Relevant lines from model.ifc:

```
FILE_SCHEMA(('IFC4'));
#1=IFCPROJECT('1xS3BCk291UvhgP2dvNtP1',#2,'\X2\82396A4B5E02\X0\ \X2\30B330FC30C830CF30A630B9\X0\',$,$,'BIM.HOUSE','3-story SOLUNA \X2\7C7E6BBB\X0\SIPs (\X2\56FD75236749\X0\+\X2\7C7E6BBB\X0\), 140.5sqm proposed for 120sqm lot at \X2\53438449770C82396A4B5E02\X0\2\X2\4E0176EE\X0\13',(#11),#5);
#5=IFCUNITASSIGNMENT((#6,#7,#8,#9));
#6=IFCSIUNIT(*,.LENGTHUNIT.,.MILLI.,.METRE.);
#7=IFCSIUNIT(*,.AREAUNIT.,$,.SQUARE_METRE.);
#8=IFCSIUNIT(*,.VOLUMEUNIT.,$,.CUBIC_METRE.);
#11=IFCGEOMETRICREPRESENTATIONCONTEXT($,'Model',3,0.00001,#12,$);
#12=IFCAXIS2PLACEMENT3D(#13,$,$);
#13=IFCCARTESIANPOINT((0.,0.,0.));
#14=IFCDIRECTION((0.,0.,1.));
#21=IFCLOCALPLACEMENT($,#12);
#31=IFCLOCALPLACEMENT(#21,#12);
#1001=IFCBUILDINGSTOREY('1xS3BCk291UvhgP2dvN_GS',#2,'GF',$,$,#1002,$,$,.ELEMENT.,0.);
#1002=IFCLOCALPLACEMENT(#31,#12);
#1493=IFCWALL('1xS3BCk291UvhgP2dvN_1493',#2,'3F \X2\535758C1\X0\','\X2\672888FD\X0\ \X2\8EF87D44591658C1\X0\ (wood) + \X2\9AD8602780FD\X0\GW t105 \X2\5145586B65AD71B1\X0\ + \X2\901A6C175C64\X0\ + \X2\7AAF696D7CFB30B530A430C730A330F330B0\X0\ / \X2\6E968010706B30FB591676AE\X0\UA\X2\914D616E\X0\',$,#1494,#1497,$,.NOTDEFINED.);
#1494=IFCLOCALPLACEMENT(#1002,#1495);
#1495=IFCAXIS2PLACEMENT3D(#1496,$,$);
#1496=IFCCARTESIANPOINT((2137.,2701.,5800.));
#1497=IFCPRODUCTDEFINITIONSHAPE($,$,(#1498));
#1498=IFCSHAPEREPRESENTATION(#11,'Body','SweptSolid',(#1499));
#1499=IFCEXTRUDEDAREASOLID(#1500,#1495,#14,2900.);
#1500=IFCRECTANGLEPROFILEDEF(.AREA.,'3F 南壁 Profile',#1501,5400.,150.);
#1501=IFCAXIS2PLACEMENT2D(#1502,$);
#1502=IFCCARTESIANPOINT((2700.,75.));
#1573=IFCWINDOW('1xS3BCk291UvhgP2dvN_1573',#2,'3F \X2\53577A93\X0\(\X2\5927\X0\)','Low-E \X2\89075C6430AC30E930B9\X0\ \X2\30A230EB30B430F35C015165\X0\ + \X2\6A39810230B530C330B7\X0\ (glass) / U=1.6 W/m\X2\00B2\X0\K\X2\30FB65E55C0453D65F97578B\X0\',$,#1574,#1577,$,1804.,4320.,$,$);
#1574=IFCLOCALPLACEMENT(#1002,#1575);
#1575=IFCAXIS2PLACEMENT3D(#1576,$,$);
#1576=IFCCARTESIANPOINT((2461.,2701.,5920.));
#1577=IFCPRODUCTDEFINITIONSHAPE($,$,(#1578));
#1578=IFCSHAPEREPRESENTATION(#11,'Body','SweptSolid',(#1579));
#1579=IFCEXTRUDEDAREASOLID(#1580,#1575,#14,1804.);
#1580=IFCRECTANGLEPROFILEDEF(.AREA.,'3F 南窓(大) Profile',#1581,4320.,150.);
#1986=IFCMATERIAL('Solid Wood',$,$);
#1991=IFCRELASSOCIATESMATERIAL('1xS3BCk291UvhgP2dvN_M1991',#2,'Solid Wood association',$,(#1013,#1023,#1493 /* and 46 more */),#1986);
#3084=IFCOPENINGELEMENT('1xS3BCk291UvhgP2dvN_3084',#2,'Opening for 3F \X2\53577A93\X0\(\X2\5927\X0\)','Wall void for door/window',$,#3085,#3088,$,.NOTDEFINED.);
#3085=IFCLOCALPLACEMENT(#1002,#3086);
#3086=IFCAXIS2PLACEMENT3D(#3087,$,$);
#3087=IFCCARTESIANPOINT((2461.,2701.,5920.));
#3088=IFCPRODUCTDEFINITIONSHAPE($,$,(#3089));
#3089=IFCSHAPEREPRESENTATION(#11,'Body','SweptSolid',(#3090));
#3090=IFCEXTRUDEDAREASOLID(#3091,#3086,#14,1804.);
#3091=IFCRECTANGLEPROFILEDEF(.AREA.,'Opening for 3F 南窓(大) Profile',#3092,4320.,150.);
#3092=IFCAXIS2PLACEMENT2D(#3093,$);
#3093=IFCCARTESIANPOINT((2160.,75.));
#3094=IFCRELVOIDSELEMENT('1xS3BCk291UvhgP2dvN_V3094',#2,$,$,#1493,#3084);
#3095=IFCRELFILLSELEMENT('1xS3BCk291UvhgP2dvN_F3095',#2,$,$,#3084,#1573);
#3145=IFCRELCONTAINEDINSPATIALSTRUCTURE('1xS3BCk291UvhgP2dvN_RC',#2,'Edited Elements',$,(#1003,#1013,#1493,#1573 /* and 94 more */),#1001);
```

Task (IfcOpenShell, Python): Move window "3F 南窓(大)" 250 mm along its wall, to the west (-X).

```python
import ifcopenshell
import ifcopenshell.api.geometry
import ifcopenshell.util.placement
import ifcopenshell.util.unit

model = ifcopenshell.open("model.ifc")
unit_scale = ifcopenshell.util.unit.calculate_unit_scale(model)

window = model.by_id(1573)
opening = window.FillsVoids[0].RelatingOpeningElement
wall = opening.VoidsElements[0].RelatingBuildingElement

wall_matrix = ifcopenshell.util.placement.get_local_placement(wall.ObjectPlacement)
shift = wall_matrix[:3, 0] * -0.25 / unit_scale
before = ifcopenshell.util.placement.get_local_placement(window.ObjectPlacement)[:3, 3].copy()

# The window is not placed relative to its opening, so move both.
for product in (opening, window):
    matrix = ifcopenshell.util.placement.get_local_placement(product.ObjectPlacement)
    matrix[:3, 3] += shift
    ifcopenshell.api.geometry.edit_object_placement(model, product=product, matrix=matrix, is_si=False)

after = ifcopenshell.util.placement.get_local_placement(window.ObjectPlacement)[:3, 3]
print("window moved by", (after - before).round(3) + 0.0)

model.write("model_v2.ifc")
```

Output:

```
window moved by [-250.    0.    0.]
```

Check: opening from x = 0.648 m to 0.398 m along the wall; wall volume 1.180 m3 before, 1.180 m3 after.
